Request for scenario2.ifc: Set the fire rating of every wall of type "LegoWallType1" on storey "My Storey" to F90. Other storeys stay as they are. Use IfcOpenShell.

First a look at what the model holds.

```python
import ifcopenshell
import ifcopenshell.util.element

model = ifcopenshell.open("scenario2.ifc")
print(model.schema)
storey = next(s for s in model.by_type("IfcBuildingStorey") if s.Name == "My Storey")
walls = [e for e in ifcopenshell.util.element.get_decomposition(storey) if e.is_a("IfcWall")]
seen = {}
for e in walls:
    element_type = ifcopenshell.util.element.get_type(e)
    key = (element_type.Name if element_type != e and element_type else None, ifcopenshell.util.element.get_pset(e, "Pset_WallCommon", "FireRating"))
    seen[key] = seen.get(key, 0) + 1
for (name, value), count in sorted(seen.items(), key=str):
    print(count, "x", name, "|", value)
```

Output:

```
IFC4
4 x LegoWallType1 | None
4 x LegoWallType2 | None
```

```python
import ifcopenshell
import ifcopenshell.api.pset
import ifcopenshell.util.element

model = ifcopenshell.open("scenario2.ifc")

storey = next(s for s in model.by_type("IfcBuildingStorey") if s.Name == "My Storey")
walls = [e for e in ifcopenshell.util.element.get_decomposition(storey) if e.is_a("IfcWall")]

count = 0
for e in walls:
    element_type = ifcopenshell.util.element.get_type(e)
    if element_type in (None, e) or element_type.Name != "LegoWallType1":
        continue
    # add_pset returns the element's existing set when there is one.
    pset = ifcopenshell.api.pset.add_pset(model, product=e, name="Pset_WallCommon")
    ifcopenshell.api.pset.edit_pset(model, pset=pset, properties={"FireRating": "F90"})
    count += 1

print(count, "walls updated")

model.write("scenario2_v2.ifc")
```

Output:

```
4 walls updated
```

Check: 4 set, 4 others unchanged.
